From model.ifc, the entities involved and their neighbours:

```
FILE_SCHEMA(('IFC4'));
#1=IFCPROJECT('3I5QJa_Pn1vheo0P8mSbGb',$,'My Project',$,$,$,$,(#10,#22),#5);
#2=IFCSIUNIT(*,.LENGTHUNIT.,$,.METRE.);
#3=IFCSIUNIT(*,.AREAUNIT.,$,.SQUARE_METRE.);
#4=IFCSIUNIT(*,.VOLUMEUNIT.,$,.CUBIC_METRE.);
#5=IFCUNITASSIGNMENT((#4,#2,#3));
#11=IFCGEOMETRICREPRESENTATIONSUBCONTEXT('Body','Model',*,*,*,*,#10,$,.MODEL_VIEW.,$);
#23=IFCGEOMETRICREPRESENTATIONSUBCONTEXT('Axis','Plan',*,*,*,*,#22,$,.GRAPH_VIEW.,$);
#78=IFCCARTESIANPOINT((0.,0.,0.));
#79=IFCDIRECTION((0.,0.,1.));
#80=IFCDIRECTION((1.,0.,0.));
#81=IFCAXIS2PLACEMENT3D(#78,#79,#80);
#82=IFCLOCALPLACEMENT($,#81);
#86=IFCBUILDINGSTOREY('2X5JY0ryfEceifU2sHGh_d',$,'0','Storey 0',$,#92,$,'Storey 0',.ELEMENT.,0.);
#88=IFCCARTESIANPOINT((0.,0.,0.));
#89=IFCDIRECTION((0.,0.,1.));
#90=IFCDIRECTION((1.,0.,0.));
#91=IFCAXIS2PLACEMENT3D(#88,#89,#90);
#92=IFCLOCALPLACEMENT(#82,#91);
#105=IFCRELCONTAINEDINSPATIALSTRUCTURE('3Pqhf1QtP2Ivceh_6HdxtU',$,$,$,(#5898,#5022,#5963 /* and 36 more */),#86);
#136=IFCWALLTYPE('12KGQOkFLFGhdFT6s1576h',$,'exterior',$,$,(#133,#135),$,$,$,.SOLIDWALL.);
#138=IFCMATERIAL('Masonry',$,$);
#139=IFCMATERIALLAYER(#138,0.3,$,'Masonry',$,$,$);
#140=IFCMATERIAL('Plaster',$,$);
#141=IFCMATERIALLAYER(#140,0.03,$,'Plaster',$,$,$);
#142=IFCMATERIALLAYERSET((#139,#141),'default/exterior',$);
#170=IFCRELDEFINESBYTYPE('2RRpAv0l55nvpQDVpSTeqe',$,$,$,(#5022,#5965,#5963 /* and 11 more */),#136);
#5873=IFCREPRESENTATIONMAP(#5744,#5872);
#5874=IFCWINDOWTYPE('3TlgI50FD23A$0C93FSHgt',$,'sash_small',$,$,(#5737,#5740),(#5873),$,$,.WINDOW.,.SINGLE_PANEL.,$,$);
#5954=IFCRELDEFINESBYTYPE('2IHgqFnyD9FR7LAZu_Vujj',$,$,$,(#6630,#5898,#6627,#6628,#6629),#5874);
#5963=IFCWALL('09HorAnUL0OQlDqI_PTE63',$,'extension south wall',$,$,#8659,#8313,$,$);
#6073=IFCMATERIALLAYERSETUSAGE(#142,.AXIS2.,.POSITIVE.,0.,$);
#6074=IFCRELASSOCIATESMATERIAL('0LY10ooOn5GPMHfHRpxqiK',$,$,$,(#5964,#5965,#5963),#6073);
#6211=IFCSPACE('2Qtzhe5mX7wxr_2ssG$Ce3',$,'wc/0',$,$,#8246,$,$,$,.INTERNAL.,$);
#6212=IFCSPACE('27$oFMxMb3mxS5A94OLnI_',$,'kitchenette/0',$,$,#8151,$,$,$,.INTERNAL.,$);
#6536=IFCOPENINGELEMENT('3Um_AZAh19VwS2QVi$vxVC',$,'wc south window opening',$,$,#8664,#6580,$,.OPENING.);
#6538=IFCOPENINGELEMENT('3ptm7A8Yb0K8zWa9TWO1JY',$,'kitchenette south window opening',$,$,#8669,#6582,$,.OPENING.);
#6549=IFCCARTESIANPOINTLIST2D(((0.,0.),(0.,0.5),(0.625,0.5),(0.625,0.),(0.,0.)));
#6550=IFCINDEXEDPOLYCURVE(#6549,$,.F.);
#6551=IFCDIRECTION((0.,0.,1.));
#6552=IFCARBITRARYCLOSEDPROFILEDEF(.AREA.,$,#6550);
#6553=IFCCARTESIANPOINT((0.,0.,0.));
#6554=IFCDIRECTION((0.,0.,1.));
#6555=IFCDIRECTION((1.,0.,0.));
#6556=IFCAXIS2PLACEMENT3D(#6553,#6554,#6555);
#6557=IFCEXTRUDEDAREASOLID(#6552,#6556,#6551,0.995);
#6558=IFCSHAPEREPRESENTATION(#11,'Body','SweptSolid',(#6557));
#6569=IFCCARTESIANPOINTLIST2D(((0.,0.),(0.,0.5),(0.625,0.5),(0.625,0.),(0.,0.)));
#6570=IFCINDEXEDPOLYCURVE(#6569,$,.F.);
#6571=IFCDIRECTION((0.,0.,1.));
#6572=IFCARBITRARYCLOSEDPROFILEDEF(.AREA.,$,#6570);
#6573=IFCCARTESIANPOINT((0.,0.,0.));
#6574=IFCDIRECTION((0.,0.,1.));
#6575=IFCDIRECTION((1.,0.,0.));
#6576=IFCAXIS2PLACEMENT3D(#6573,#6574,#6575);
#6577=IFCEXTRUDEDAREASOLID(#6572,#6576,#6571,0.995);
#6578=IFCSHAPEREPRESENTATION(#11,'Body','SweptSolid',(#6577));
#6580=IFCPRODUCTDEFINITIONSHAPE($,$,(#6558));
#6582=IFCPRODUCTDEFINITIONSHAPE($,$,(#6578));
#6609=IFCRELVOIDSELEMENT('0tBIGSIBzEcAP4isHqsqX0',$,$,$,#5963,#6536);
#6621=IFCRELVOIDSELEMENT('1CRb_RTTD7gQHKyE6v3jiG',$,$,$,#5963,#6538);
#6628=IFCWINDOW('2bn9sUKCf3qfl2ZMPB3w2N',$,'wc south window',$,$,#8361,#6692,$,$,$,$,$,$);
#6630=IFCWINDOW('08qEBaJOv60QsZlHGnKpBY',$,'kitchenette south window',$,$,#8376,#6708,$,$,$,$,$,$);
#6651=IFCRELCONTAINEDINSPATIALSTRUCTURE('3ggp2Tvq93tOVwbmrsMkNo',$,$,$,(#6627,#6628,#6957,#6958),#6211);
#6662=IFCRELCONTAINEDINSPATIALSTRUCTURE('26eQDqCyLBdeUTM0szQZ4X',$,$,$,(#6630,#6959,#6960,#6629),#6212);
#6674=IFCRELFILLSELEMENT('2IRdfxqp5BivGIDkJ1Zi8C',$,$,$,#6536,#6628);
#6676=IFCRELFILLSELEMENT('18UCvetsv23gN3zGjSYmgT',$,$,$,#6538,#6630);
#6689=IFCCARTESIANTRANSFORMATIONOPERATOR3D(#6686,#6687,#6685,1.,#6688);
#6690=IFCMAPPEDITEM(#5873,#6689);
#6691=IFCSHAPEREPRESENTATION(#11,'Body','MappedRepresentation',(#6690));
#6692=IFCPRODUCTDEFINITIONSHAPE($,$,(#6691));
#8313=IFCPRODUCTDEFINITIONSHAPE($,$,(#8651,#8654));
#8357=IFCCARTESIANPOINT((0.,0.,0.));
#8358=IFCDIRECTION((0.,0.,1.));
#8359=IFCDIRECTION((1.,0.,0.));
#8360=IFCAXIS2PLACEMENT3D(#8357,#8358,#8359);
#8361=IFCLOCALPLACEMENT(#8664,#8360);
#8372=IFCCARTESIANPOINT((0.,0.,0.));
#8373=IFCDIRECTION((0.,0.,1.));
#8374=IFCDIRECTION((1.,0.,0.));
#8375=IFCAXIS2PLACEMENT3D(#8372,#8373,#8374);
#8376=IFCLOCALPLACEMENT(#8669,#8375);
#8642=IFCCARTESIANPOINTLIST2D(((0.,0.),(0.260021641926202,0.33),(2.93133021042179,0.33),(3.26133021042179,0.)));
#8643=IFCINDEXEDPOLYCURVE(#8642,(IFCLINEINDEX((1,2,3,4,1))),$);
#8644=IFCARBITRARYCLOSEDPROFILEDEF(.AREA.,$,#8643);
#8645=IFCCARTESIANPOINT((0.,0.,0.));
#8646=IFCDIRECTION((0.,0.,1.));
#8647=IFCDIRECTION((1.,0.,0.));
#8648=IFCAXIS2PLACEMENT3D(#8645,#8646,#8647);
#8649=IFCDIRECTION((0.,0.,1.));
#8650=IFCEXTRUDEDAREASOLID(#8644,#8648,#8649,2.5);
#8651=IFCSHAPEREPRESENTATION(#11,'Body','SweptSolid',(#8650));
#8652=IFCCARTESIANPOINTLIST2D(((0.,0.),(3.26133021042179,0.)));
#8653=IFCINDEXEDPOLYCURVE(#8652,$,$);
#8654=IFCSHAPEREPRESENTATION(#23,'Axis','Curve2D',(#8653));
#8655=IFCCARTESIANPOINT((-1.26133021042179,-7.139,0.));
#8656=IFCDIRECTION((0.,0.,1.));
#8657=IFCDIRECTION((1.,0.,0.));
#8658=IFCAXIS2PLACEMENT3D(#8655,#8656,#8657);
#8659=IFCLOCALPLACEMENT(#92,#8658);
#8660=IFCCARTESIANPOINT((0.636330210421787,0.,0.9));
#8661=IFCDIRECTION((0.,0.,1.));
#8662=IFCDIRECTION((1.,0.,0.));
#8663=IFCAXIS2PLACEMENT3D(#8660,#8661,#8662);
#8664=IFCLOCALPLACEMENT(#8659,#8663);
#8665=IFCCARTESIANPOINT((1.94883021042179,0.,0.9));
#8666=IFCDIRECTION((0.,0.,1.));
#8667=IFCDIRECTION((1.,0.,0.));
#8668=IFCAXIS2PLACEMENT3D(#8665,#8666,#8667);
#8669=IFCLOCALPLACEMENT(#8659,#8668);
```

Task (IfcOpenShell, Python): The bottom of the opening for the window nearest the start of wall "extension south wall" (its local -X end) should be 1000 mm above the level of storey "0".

```python
import numpy as np
import ifcopenshell
import ifcopenshell.api.geometry
import ifcopenshell.geom
import ifcopenshell.util.element
import ifcopenshell.util.placement
import ifcopenshell.util.shape
import ifcopenshell.util.unit

model = ifcopenshell.open("model.ifc")
unit_scale = ifcopenshell.util.unit.calculate_unit_scale(model)

window = model.by_guid("2bn9sUKCf3qfl2ZMPB3w2N")
opening = window.FillsVoids[0].RelatingOpeningElement
storey = ifcopenshell.util.element.get_container(window, ifc_class="IfcBuildingStorey")
level = ifcopenshell.util.placement.get_local_placement(storey.ObjectPlacement)[2, 3]

# The opening's origin need not be at the sill, so measure its lowest point.
shape = ifcopenshell.geom.create_shape(ifcopenshell.geom.settings(), opening)
bottom = ifcopenshell.util.shape.get_shape_bottom_elevation(shape, shape.geometry) / unit_scale
dz = level + 1 / unit_scale - bottom

shift = np.array([0.0, 0.0, dz])
# The window is placed relative to its opening, so it follows when the opening moves.
matrix = ifcopenshell.util.placement.get_local_placement(opening.ObjectPlacement)
matrix[:3, 3] += shift
ifcopenshell.api.geometry.edit_object_placement(
    model, product=opening, matrix=matrix, is_si=False, should_transform_children=True
)

print(f"moved by {dz * unit_scale:+.3f} m")

model.write("model_edited.ifc")
```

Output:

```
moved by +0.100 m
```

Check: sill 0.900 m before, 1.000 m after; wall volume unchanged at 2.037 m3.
